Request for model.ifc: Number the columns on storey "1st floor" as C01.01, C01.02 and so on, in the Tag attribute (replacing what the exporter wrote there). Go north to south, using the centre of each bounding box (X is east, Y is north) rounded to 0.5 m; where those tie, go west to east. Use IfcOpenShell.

First a look at what the model holds.

```python
import ifcopenshell
import ifcopenshell.util.element
import ifcopenshell.util.placement

model = ifcopenshell.open("model.ifc")
print(model.schema)
storey = next(s for s in model.by_type("IfcBuildingStorey") if s.Name == "1st floor")
columns = [e for e in ifcopenshell.util.element.get_decomposition(storey) if e.is_a("IfcColumn")]
for e in sorted(columns, key=lambda e: e.id()):
    origin = ifcopenshell.util.placement.get_local_placement(e.ObjectPlacement)[:3, 3]
    print(e.id(), e.Tag, e.Name, origin.round(2) + 0.0, sep=" | ")
```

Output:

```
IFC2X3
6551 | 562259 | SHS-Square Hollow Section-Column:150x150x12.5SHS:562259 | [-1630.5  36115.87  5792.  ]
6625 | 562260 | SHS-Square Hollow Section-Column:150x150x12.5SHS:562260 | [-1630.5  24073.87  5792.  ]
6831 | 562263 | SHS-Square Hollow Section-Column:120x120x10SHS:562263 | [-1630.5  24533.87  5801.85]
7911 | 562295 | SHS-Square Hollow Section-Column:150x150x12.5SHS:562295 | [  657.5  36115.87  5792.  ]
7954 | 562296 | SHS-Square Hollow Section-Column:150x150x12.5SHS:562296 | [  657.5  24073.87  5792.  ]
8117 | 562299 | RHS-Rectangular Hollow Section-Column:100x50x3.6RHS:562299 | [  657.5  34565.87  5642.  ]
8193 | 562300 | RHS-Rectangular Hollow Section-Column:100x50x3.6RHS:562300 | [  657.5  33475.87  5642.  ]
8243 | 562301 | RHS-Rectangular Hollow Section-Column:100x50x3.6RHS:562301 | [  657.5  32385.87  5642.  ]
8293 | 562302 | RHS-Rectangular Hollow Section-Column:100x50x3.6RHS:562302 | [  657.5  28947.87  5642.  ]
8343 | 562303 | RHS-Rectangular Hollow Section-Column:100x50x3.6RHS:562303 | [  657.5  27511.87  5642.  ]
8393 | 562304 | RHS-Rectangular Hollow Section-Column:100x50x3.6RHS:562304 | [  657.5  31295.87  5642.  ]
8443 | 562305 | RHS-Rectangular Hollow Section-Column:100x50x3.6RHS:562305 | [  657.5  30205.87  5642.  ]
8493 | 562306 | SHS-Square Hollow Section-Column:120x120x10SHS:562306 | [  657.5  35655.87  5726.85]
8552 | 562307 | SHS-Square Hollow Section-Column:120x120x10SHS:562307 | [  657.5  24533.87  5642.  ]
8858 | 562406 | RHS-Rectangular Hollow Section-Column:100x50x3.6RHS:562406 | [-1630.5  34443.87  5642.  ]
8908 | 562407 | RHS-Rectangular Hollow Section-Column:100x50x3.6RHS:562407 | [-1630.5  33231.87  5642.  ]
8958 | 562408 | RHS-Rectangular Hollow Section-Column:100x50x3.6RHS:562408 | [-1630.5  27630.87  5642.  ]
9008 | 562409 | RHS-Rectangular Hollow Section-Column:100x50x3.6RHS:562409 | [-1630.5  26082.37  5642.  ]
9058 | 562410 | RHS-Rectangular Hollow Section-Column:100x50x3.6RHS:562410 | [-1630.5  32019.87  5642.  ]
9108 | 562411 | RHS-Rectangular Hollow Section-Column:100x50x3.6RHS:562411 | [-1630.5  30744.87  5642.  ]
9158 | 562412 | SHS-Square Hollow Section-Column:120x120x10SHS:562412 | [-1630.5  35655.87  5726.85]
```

```python
import ifcopenshell
import ifcopenshell.geom
import ifcopenshell.util.element
import ifcopenshell.util.shape

model = ifcopenshell.open("model.ifc")
settings = ifcopenshell.geom.settings()
settings.set("use-world-coords", True)


def centre(element):
    shape = ifcopenshell.geom.create_shape(settings, element)
    return ifcopenshell.util.shape.get_bbox_centroid(shape.geometry)


storey = next(s for s in model.by_type("IfcBuildingStorey") if s.Name == "1st floor")
columns = [e for e in ifcopenshell.util.element.get_decomposition(storey) if e.is_a("IfcColumn")]

# Insertion points can sit at a corner or the storey origin, so sort by the geometry (in metres).
centres = {e: centre(e) for e in columns}
columns.sort(key=lambda e: (-round(centres[e][1] / 0.5), centres[e][0]))

for i, e in enumerate(columns, start=1):
    number = f"C01.{i:02d}"
    e.Tag = number
    print(e.id(), number)

model.write("model_edited.ifc")
```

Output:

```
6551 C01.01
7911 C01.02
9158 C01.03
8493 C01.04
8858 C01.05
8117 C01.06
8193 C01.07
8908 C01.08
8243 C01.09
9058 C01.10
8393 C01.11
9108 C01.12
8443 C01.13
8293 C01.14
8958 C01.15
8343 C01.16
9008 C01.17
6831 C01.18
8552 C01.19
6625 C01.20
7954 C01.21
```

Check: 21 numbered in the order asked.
